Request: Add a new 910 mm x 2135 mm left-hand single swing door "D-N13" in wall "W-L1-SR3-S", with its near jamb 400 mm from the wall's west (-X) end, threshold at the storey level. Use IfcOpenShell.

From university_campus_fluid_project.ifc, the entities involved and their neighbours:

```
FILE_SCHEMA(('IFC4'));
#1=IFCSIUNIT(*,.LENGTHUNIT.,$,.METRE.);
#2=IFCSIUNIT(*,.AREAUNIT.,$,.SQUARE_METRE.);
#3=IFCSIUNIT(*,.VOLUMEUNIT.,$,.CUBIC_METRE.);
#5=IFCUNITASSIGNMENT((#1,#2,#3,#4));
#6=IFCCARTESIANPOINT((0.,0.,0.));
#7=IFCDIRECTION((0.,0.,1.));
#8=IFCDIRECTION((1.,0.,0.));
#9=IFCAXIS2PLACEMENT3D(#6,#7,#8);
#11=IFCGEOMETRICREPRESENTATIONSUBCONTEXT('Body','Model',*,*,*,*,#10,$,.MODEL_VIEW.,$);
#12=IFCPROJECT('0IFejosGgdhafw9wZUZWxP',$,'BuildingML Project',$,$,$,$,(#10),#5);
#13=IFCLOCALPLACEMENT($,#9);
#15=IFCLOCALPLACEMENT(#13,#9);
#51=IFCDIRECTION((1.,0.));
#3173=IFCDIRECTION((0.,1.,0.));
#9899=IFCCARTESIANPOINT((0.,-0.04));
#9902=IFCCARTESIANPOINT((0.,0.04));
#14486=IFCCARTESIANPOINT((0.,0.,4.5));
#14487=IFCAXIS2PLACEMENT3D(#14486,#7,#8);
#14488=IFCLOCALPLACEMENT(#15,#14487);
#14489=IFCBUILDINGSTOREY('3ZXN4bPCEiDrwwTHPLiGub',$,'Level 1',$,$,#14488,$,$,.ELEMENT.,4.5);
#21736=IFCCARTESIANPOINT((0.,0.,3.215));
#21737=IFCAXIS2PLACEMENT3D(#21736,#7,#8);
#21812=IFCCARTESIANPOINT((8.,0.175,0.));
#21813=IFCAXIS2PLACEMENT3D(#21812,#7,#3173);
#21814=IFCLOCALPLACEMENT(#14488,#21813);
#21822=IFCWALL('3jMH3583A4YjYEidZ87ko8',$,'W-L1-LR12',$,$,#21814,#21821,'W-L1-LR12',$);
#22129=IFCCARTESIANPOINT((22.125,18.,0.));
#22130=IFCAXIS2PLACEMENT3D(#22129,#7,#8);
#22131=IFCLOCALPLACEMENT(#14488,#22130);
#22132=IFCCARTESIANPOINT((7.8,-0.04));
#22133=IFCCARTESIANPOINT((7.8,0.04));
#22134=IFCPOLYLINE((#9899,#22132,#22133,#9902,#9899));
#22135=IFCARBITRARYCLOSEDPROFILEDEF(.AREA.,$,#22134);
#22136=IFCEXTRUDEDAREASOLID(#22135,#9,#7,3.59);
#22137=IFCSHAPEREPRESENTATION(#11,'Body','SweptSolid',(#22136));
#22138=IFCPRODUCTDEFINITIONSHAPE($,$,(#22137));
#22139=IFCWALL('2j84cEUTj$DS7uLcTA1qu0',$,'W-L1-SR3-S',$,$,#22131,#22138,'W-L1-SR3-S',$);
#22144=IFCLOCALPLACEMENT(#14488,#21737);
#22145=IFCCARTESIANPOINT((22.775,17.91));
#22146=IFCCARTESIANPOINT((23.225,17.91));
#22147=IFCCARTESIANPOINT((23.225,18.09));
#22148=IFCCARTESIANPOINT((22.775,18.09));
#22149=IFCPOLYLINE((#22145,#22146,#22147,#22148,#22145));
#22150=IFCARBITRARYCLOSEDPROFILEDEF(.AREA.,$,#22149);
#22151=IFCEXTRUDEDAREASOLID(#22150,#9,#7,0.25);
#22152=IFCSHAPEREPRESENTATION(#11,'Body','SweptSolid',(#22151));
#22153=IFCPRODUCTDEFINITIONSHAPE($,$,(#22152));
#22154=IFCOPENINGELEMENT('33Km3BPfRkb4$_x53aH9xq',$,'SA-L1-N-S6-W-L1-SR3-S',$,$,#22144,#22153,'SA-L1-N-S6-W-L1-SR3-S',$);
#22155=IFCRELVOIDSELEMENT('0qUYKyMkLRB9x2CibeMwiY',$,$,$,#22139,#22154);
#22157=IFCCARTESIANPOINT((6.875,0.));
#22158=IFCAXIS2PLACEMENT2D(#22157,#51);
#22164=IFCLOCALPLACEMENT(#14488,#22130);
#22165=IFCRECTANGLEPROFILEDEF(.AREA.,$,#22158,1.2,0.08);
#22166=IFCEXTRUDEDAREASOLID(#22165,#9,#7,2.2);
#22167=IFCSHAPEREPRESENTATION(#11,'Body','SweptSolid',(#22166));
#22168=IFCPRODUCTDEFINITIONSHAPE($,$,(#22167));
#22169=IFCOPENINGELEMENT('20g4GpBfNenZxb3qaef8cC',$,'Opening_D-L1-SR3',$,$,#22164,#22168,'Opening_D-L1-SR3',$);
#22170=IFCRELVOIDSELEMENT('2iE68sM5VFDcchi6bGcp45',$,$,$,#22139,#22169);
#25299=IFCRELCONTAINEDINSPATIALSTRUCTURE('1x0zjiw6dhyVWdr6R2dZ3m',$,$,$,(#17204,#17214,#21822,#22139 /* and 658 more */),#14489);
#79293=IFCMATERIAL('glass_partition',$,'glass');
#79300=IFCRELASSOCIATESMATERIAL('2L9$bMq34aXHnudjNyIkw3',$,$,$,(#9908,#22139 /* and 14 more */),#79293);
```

```python
import numpy as np
import ifcopenshell
import ifcopenshell.api.feature
import ifcopenshell.api.geometry
import ifcopenshell.api.root
import ifcopenshell.api.spatial
import ifcopenshell.geom
import ifcopenshell.util.element
import ifcopenshell.util.placement
import ifcopenshell.util.representation
import ifcopenshell.util.shape
import ifcopenshell.util.unit

model = ifcopenshell.open("university_campus_fluid_project.ifc")
unit_scale = ifcopenshell.util.unit.calculate_unit_scale(model)
settings = ifcopenshell.geom.settings()


def volume(element):
    """Net volume in cubic metres, openings subtracted."""
    shape = ifcopenshell.geom.create_shape(settings, element)
    return ifcopenshell.util.shape.get_volume(shape.geometry)


wall = model.by_guid("2j84cEUTj$DS7uLcTA1qu0")
storey = ifcopenshell.util.element.get_container(wall, ifc_class="IfcBuildingStorey")
context = ifcopenshell.util.representation.get_context(model, "Model", "Body", "MODEL_VIEW")
before = volume(wall)

width, height, from_end, sill = 0.91, 2.135, 0.4, 0.0  # metres

# The wall runs along its own X axis, and the end named is its -X end.
wall_shape = ifcopenshell.geom.create_shape(settings, wall)
x, y, z = ifcopenshell.util.shape.get_vertices(wall_shape.geometry).T
start = x.min() + from_end
face, thickness = float(y.min()), float(y.max() - y.min())
wall_matrix = ifcopenshell.util.placement.get_local_placement(wall.ObjectPlacement)
level = ifcopenshell.util.placement.get_local_placement(storey.ObjectPlacement)[2, 3]


def in_wall(x, y):
    """Placement at x, y metres in the wall's axes, at sill height."""
    matrix = wall_matrix.copy()
    matrix[:, 3] = wall_matrix @ np.array([x / unit_scale, y / unit_scale, 0.0, 1.0])
    matrix[2, 3] = level + sill / unit_scale
    return matrix


# Opening: a box that overshoots both wall faces by 50 mm.
opening = ifcopenshell.api.root.create_entity(model, ifc_class="IfcOpeningElement", predefined_type="OPENING")
box = ifcopenshell.api.geometry.add_wall_representation(
    model, context=context, length=width, height=height, thickness=thickness + 0.1
)
ifcopenshell.api.geometry.assign_representation(model, product=opening, representation=box)
ifcopenshell.api.geometry.edit_object_placement(model, product=opening, matrix=in_wall(start, face - 0.05), is_si=False)
ifcopenshell.api.feature.add_feature(model, feature=opening, element=wall)

door = ifcopenshell.api.root.create_entity(model, ifc_class="IfcDoor", name="D-N13", predefined_type="DOOR")
door.OverallWidth, door.OverallHeight = width / unit_scale, height / unit_scale
door.OperationType = "SINGLE_SWING_LEFT"
body = ifcopenshell.api.geometry.add_door_representation(
    model,
    context=context,
    overall_width=door.OverallWidth,
    overall_height=door.OverallHeight,
    operation_type="SINGLE_SWING_LEFT",
    lining_properties={"LiningDepth": thickness / unit_scale, "ThresholdDepth": thickness / unit_scale},
)
ifcopenshell.api.geometry.assign_representation(model, product=door, representation=body)
ifcopenshell.api.spatial.assign_container(model, products=[door], relating_structure=storey)
ifcopenshell.api.feature.add_filling(model, opening=opening, element=door)

# The lining spans the wall, so the door starts at the wall face.
ifcopenshell.api.geometry.edit_object_placement(model, product=door, matrix=in_wall(start, face), is_si=False)

after = volume(wall)

print(f"wall volume {before:.3f} -> {after:.3f} m3")

model.write("university_campus_fluid_project-out.ifc")
```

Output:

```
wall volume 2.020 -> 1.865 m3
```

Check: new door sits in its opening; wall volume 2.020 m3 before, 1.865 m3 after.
